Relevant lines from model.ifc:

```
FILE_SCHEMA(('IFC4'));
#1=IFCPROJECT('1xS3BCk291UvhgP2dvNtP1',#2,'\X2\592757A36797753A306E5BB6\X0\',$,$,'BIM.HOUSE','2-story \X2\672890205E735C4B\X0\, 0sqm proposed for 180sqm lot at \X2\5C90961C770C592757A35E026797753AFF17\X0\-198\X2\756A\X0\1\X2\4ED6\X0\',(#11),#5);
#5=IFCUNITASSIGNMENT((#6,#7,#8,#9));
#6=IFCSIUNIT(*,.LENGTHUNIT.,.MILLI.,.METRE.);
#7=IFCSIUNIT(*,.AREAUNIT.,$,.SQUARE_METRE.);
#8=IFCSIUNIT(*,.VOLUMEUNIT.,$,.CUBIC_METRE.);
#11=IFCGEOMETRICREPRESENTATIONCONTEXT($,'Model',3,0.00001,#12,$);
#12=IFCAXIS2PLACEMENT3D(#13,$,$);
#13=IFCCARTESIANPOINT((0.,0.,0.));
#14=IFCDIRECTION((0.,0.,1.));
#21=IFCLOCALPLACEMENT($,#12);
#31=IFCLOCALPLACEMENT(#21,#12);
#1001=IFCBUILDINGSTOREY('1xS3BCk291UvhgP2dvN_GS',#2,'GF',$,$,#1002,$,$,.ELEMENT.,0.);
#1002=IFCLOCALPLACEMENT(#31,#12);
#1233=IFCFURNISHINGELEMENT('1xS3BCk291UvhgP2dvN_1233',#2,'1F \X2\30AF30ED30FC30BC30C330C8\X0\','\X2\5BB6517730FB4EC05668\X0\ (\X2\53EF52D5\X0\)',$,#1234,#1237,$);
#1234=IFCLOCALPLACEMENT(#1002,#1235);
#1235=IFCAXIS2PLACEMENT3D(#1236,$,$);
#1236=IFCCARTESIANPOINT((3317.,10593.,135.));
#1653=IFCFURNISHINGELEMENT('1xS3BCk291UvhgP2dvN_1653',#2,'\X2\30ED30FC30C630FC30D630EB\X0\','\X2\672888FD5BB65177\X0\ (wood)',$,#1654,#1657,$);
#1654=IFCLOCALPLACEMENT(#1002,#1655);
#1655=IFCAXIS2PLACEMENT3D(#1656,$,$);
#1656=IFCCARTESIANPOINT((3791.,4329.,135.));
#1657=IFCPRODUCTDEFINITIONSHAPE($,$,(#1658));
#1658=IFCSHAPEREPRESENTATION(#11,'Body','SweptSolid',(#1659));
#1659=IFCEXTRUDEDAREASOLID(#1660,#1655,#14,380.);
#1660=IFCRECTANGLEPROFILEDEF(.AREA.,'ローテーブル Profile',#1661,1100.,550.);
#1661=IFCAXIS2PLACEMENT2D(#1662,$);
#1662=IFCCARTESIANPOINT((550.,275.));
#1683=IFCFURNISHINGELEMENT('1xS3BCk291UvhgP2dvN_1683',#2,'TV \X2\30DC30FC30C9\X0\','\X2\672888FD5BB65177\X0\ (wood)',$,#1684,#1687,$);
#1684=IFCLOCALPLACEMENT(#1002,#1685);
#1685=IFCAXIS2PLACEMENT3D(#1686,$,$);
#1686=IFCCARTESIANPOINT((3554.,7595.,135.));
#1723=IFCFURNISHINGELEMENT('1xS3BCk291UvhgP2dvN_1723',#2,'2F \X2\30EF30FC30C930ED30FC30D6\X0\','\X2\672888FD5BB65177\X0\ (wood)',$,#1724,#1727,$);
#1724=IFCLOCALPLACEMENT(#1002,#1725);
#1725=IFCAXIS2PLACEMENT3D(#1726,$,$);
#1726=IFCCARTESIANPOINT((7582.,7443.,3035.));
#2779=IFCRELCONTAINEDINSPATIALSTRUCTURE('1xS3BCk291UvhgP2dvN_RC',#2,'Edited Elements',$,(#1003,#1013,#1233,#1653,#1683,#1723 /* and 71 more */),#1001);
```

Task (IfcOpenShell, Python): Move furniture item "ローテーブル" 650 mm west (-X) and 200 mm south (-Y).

```python
import ifcopenshell
import ifcopenshell.api.geometry
import ifcopenshell.util.placement

model = ifcopenshell.open("model.ifc")

item = model.by_id(1653)
matrix = ifcopenshell.util.placement.get_local_placement(item.ObjectPlacement)
matrix[0, 3] -= 650.0
matrix[1, 3] -= 200.0
ifcopenshell.api.geometry.edit_object_placement(model, product=item, matrix=matrix, is_si=False)

print(ifcopenshell.util.placement.get_local_placement(item.ObjectPlacement).round(3) + 0.0)

model.write("model_edited.ifc")
```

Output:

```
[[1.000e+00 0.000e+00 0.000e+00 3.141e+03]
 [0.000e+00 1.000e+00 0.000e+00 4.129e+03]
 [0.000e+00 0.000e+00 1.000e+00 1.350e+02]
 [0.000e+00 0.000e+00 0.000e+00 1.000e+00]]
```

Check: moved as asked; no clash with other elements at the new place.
